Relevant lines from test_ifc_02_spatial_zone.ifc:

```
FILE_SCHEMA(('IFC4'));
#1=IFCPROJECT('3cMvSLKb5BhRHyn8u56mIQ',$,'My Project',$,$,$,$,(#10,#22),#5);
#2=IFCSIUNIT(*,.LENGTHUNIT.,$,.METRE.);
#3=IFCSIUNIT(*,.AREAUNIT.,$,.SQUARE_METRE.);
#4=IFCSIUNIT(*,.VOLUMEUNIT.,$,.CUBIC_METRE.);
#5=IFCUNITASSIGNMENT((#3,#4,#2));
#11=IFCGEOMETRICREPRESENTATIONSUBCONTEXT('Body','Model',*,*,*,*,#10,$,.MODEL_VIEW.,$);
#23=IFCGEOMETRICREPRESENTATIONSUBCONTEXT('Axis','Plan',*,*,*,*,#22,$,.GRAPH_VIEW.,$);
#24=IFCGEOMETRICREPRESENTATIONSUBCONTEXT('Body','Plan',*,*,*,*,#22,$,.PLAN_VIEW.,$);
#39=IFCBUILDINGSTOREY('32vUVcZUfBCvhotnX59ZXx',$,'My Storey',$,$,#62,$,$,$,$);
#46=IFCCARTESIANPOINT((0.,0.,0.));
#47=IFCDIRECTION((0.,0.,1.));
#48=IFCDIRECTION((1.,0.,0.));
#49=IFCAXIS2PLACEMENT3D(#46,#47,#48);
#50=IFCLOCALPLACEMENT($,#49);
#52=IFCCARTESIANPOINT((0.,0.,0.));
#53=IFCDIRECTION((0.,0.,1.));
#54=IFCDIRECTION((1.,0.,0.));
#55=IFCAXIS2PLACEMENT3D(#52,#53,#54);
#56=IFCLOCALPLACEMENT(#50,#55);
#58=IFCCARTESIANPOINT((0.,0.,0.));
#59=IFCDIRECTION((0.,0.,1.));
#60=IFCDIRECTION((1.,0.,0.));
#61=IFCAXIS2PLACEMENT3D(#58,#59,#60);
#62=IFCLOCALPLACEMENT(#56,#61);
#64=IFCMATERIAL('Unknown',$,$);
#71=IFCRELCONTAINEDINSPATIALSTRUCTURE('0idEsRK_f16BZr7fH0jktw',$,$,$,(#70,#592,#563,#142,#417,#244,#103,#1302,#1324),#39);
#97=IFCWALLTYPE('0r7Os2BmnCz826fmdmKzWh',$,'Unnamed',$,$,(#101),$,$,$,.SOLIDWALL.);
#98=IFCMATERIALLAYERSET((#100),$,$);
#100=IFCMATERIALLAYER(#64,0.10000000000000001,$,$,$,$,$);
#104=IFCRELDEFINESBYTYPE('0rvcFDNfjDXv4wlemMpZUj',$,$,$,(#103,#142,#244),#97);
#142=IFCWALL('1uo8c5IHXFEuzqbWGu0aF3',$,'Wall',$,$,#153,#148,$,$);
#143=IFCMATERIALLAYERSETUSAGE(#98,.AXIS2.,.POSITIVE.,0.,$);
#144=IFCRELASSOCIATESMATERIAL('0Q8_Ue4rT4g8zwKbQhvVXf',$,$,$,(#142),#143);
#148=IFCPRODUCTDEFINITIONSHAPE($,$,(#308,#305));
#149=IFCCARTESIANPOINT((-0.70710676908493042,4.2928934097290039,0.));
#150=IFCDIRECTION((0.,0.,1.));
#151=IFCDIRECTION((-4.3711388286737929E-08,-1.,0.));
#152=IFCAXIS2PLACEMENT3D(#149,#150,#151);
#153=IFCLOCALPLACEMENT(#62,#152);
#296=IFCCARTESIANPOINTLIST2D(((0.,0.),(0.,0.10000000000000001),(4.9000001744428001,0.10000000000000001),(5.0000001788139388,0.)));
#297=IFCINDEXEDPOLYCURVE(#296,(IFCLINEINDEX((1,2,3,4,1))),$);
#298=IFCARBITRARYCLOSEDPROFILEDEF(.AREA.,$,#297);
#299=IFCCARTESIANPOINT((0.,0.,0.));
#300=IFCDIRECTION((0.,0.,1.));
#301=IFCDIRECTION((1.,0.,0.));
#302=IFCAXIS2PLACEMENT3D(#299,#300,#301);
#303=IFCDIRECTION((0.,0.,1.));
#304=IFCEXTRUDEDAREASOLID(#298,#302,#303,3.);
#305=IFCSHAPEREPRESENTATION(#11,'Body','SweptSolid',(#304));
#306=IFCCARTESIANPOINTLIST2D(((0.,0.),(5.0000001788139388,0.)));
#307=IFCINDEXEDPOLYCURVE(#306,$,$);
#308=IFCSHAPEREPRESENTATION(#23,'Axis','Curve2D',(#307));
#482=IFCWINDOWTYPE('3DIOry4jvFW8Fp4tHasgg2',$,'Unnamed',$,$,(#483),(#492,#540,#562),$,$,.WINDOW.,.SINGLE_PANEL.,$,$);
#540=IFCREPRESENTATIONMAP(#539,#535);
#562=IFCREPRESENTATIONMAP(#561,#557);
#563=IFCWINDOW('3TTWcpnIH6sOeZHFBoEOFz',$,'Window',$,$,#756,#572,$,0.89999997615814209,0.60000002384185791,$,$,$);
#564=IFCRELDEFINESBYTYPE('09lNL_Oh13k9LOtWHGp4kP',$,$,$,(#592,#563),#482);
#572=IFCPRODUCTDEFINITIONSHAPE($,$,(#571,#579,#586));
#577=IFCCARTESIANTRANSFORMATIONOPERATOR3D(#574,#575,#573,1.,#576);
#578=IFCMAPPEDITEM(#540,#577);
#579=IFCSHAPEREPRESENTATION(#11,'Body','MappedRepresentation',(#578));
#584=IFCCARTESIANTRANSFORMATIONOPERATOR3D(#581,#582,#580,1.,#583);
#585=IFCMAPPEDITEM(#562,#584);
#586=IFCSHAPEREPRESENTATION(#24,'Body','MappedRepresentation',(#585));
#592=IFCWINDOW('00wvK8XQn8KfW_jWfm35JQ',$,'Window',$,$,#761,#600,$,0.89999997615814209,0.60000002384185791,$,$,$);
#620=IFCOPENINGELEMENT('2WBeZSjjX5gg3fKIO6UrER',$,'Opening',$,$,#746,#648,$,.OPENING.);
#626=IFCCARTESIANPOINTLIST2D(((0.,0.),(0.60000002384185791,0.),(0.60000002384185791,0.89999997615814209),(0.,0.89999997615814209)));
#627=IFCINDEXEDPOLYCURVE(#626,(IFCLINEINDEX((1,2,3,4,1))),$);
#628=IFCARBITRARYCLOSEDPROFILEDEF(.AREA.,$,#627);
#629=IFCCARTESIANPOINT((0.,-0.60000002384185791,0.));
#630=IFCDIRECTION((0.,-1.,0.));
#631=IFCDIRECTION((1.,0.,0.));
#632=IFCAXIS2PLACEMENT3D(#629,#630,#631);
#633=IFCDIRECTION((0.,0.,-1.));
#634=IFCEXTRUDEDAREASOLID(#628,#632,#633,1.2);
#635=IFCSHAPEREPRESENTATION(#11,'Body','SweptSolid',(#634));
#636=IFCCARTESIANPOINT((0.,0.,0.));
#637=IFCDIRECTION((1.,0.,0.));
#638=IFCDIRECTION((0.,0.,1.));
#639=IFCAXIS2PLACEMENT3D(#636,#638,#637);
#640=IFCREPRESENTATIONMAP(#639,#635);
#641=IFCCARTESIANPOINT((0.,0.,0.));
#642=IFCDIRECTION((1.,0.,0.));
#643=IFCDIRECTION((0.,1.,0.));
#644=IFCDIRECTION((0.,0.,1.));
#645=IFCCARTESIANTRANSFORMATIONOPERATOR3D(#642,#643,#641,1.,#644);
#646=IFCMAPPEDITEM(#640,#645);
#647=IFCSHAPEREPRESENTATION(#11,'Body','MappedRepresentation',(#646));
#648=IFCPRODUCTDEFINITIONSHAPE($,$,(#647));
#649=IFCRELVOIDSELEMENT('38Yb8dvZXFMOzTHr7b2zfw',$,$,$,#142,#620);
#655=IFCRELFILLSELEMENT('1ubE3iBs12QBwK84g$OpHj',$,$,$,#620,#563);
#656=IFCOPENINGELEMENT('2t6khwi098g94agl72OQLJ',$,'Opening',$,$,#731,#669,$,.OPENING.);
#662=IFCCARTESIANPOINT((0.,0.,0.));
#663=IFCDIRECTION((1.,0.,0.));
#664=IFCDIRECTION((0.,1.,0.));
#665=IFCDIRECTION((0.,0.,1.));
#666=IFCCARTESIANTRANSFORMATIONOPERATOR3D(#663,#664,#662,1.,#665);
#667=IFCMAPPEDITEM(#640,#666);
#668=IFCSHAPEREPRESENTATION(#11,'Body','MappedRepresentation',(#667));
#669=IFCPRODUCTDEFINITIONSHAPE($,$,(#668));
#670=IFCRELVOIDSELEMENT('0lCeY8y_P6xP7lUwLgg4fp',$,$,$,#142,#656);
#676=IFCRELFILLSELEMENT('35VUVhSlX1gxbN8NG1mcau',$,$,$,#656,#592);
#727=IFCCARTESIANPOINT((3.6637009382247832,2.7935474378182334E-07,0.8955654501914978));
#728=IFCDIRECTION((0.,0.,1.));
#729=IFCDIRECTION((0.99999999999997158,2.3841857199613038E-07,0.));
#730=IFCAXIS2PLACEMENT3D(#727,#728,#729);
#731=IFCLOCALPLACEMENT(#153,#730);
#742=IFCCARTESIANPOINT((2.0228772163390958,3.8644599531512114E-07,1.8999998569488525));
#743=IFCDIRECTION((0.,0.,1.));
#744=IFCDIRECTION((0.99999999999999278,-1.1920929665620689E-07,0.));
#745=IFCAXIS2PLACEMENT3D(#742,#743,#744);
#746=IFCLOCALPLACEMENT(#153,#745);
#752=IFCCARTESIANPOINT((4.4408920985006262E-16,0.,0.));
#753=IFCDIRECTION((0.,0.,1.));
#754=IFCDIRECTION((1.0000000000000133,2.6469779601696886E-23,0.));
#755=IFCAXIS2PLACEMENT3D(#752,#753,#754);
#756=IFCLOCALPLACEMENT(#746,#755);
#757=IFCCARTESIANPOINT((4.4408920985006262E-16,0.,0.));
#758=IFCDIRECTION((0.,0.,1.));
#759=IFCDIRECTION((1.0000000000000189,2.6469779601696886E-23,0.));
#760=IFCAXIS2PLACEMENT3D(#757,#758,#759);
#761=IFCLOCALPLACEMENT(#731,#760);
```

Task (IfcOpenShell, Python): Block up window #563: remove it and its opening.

```python
import ifcopenshell
import ifcopenshell.api.feature
import ifcopenshell.api.root
import ifcopenshell.geom
import ifcopenshell.util.shape

model = ifcopenshell.open("test_ifc_02_spatial_zone.ifc")
settings = ifcopenshell.geom.settings()


def volume(element):
    """Net volume in cubic metres, openings subtracted."""
    shape = ifcopenshell.geom.create_shape(settings, element)
    return ifcopenshell.util.shape.get_volume(shape.geometry)


window = model.by_id(563)
opening = window.FillsVoids[0].RelatingOpeningElement
wall = opening.VoidsElements[0].RelatingBuildingElement
before = volume(wall)

ifcopenshell.api.root.remove_product(model, product=window)
ifcopenshell.api.feature.remove_feature(model, feature=opening)

after = volume(wall)

print(f"wall volume {before:.3f} -> {after:.3f} m3")

model.write("test_ifc_02_spatial_zone_v2.ifc")
```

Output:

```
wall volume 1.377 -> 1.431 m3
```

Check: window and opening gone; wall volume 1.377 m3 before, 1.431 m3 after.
